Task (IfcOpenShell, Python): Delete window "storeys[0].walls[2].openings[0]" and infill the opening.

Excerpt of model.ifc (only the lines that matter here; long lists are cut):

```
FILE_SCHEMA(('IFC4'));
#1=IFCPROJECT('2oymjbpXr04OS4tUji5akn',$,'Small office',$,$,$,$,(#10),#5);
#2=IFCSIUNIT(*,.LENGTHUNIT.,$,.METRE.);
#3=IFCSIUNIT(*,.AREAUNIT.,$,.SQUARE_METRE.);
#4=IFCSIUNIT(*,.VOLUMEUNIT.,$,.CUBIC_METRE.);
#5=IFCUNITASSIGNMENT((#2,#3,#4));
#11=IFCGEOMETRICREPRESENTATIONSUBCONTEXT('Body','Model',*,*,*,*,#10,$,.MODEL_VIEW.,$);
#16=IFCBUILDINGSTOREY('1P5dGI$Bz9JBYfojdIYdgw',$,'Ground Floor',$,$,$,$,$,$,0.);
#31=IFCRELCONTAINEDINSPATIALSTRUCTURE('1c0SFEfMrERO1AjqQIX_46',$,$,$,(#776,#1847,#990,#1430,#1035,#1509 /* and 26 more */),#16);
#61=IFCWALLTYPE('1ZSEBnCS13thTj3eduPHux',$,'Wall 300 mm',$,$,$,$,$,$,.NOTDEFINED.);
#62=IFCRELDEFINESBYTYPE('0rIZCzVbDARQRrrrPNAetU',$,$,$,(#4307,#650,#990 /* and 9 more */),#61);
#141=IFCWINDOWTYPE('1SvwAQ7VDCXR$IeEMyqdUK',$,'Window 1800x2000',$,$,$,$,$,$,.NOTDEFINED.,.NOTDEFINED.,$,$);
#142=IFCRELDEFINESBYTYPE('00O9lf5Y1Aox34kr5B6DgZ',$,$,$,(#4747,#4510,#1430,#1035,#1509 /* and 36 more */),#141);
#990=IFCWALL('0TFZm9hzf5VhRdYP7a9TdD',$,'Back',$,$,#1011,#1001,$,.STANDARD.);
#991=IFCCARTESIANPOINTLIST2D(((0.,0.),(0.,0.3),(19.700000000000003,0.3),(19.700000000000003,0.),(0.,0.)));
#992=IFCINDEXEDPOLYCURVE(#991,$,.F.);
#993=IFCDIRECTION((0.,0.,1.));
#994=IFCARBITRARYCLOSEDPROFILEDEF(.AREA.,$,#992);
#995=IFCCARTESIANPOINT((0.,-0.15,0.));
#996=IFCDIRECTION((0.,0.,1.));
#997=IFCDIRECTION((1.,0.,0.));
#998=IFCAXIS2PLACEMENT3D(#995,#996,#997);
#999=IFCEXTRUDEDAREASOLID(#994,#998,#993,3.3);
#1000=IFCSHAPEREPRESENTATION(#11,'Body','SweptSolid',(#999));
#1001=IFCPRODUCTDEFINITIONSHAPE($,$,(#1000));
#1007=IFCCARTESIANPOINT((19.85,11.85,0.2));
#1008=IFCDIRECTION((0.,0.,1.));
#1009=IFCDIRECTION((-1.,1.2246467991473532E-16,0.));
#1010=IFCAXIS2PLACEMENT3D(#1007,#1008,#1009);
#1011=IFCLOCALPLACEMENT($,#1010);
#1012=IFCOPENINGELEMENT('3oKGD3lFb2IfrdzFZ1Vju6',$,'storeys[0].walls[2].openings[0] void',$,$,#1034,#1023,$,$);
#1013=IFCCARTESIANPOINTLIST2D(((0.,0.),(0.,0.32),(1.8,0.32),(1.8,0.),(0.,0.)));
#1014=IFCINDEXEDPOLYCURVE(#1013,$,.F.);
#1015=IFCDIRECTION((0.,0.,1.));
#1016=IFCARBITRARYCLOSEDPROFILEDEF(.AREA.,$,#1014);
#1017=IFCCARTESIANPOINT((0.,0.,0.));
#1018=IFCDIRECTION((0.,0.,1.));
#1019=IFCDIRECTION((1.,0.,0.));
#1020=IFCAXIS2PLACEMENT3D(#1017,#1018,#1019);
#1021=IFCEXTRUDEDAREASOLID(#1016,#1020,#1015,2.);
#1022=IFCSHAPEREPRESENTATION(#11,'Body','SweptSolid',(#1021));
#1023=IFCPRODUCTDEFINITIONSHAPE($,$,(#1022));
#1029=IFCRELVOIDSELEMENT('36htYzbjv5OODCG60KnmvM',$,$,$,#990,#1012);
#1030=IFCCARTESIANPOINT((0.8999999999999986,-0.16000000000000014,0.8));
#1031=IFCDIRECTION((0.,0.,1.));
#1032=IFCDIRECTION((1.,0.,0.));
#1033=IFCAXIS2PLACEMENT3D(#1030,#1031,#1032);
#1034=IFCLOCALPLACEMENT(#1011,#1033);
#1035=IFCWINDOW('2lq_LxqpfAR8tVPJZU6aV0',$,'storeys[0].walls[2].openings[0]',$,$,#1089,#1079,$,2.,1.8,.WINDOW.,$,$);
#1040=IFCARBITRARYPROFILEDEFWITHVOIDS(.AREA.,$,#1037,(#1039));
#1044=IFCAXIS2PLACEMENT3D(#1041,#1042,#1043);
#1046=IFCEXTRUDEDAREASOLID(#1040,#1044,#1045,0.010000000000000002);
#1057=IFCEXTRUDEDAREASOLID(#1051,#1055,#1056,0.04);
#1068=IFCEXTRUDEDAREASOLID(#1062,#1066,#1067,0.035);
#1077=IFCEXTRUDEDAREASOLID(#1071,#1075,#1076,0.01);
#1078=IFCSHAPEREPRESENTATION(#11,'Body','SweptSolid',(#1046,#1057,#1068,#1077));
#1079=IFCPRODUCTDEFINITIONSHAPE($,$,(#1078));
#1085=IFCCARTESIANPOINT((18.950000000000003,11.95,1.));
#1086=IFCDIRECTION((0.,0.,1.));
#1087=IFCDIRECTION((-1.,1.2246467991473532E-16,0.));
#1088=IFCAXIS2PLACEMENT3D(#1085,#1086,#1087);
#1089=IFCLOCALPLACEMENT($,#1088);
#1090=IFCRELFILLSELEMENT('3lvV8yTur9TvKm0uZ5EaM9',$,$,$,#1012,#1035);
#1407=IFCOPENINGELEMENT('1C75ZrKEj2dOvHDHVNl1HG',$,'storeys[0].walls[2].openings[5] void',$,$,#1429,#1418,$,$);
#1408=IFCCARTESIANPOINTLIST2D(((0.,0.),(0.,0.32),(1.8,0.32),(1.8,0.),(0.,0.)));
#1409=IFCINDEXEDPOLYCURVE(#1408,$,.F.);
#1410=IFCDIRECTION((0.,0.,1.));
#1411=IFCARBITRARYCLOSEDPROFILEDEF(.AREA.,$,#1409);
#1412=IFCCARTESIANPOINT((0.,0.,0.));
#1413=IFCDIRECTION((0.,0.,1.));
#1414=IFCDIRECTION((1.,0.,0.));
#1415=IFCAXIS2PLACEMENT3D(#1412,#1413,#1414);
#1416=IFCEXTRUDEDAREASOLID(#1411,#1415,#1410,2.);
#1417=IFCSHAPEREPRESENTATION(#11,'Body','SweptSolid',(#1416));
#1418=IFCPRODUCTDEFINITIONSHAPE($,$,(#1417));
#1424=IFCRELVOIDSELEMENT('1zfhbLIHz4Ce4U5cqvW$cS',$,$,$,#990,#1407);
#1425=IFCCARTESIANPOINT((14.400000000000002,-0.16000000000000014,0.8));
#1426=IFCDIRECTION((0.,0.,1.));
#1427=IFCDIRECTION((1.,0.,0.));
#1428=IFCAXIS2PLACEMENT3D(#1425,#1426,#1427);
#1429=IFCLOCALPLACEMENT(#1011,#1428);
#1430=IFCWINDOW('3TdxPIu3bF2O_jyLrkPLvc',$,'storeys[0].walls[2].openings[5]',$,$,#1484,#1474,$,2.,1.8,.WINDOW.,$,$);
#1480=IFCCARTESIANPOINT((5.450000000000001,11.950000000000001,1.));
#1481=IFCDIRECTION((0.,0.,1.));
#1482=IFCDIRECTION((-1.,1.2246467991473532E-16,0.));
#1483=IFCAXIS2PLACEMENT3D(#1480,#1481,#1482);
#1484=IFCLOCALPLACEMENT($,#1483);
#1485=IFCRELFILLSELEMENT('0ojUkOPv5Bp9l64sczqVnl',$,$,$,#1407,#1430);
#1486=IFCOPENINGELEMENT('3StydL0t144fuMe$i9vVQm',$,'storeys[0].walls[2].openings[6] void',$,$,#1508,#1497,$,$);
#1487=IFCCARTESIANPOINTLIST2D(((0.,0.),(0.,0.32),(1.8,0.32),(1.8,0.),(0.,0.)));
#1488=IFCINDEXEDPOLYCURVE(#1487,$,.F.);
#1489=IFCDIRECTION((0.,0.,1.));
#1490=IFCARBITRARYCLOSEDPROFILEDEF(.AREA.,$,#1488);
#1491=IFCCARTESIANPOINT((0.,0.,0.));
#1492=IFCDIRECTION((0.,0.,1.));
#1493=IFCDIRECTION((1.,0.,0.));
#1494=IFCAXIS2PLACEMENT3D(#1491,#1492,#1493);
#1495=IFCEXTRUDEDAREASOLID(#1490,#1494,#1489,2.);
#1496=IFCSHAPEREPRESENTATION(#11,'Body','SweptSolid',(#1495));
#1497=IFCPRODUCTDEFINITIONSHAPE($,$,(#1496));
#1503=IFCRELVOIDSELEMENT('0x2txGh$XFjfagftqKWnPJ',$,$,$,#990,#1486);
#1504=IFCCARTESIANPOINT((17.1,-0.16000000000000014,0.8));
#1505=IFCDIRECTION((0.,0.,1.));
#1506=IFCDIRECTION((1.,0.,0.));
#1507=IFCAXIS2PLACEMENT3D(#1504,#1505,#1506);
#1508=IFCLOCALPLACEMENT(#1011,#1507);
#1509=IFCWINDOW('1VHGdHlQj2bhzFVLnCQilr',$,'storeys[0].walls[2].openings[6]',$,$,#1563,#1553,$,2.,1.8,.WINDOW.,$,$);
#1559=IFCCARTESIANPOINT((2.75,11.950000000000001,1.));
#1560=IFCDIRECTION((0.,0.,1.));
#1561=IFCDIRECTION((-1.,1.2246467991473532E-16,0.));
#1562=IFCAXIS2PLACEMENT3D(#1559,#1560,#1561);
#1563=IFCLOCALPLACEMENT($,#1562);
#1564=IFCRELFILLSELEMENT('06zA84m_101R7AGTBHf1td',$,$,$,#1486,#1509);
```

```python
import ifcopenshell
import ifcopenshell.api.feature
import ifcopenshell.api.root
import ifcopenshell.geom
import ifcopenshell.util.shape

model = ifcopenshell.open("model.ifc")
settings = ifcopenshell.geom.settings()


def volume(element):
    """Net volume in cubic metres, openings subtracted."""
    shape = ifcopenshell.geom.create_shape(settings, element)
    return ifcopenshell.util.shape.get_volume(shape.geometry)


window = model.by_guid("2lq_LxqpfAR8tVPJZU6aV0")
opening = window.FillsVoids[0].RelatingOpeningElement
wall = opening.VoidsElements[0].RelatingBuildingElement
before = volume(wall)

ifcopenshell.api.root.remove_product(model, product=window)
ifcopenshell.api.feature.remove_feature(model, feature=opening)

after = volume(wall)

print(f"wall volume {before:.3f} -> {after:.3f} m3")

model.write("model_edited.ifc")
```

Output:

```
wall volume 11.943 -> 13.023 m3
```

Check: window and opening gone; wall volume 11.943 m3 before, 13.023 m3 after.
